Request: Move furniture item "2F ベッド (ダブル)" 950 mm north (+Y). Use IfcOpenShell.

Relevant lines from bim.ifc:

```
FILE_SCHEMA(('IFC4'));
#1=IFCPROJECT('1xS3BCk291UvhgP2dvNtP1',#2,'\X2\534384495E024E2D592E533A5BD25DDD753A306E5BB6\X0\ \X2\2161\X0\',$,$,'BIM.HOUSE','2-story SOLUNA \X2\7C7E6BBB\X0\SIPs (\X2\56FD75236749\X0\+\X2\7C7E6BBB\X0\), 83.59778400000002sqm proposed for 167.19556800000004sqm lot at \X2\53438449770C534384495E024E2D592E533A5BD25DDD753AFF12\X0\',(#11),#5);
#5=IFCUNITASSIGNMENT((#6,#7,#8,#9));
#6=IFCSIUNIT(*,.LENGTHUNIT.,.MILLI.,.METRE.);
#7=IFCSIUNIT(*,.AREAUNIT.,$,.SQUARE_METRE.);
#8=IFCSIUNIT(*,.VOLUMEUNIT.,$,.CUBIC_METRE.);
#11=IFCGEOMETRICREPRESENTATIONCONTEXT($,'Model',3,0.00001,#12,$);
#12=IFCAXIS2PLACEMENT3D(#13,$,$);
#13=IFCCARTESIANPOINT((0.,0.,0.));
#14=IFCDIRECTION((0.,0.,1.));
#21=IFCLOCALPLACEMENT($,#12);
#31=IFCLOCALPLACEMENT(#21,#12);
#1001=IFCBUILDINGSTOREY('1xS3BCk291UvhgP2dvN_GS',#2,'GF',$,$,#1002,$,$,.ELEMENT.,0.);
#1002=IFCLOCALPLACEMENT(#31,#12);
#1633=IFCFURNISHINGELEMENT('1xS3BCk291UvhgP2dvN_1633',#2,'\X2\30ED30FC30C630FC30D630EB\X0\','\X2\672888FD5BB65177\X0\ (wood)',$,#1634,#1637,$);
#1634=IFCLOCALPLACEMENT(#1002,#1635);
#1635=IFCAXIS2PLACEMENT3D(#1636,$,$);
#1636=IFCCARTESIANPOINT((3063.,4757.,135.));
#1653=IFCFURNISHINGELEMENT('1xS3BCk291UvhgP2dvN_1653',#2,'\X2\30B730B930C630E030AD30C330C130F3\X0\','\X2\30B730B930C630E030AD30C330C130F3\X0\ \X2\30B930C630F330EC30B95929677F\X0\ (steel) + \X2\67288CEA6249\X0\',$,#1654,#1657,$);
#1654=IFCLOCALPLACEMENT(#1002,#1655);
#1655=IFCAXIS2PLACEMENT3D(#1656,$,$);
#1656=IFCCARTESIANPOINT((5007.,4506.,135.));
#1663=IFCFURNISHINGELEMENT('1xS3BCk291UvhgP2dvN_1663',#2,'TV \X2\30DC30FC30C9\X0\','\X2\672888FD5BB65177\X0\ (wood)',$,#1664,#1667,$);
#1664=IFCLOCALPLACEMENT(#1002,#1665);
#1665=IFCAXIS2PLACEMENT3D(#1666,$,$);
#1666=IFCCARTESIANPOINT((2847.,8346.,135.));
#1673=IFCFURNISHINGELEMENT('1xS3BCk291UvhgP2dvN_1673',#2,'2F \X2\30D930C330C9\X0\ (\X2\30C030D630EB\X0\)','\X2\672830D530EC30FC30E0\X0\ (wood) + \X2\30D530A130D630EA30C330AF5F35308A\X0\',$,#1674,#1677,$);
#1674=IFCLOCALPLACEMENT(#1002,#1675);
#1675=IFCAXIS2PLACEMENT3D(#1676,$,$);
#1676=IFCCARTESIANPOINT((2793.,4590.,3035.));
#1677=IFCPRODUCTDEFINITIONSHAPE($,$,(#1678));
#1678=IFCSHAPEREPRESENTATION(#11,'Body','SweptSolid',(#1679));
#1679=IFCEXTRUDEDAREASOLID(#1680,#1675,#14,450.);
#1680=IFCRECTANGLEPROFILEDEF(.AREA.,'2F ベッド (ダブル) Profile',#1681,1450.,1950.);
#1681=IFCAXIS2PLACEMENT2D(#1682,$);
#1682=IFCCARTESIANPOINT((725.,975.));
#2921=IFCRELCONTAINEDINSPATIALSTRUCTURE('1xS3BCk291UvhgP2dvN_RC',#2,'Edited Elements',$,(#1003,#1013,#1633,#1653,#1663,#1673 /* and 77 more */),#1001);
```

```python
import ifcopenshell
import ifcopenshell.api.geometry
import ifcopenshell.util.placement
import ifcopenshell.util.unit

model = ifcopenshell.open("bim.ifc")
unit_scale = ifcopenshell.util.unit.calculate_unit_scale(model)

item = model.by_guid("1xS3BCk291UvhgP2dvN_1673")
matrix = ifcopenshell.util.placement.get_local_placement(item.ObjectPlacement)
matrix[1, 3] += 0.95 / unit_scale
ifcopenshell.api.geometry.edit_object_placement(model, product=item, matrix=matrix, is_si=False)

print(ifcopenshell.util.placement.get_local_placement(item.ObjectPlacement).round(3) + 0.0)

model.write("bim_edited.ifc")
```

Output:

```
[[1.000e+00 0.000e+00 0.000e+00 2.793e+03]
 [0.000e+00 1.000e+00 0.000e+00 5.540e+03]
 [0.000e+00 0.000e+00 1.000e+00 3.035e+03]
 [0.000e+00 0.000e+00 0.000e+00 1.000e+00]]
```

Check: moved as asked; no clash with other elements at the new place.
